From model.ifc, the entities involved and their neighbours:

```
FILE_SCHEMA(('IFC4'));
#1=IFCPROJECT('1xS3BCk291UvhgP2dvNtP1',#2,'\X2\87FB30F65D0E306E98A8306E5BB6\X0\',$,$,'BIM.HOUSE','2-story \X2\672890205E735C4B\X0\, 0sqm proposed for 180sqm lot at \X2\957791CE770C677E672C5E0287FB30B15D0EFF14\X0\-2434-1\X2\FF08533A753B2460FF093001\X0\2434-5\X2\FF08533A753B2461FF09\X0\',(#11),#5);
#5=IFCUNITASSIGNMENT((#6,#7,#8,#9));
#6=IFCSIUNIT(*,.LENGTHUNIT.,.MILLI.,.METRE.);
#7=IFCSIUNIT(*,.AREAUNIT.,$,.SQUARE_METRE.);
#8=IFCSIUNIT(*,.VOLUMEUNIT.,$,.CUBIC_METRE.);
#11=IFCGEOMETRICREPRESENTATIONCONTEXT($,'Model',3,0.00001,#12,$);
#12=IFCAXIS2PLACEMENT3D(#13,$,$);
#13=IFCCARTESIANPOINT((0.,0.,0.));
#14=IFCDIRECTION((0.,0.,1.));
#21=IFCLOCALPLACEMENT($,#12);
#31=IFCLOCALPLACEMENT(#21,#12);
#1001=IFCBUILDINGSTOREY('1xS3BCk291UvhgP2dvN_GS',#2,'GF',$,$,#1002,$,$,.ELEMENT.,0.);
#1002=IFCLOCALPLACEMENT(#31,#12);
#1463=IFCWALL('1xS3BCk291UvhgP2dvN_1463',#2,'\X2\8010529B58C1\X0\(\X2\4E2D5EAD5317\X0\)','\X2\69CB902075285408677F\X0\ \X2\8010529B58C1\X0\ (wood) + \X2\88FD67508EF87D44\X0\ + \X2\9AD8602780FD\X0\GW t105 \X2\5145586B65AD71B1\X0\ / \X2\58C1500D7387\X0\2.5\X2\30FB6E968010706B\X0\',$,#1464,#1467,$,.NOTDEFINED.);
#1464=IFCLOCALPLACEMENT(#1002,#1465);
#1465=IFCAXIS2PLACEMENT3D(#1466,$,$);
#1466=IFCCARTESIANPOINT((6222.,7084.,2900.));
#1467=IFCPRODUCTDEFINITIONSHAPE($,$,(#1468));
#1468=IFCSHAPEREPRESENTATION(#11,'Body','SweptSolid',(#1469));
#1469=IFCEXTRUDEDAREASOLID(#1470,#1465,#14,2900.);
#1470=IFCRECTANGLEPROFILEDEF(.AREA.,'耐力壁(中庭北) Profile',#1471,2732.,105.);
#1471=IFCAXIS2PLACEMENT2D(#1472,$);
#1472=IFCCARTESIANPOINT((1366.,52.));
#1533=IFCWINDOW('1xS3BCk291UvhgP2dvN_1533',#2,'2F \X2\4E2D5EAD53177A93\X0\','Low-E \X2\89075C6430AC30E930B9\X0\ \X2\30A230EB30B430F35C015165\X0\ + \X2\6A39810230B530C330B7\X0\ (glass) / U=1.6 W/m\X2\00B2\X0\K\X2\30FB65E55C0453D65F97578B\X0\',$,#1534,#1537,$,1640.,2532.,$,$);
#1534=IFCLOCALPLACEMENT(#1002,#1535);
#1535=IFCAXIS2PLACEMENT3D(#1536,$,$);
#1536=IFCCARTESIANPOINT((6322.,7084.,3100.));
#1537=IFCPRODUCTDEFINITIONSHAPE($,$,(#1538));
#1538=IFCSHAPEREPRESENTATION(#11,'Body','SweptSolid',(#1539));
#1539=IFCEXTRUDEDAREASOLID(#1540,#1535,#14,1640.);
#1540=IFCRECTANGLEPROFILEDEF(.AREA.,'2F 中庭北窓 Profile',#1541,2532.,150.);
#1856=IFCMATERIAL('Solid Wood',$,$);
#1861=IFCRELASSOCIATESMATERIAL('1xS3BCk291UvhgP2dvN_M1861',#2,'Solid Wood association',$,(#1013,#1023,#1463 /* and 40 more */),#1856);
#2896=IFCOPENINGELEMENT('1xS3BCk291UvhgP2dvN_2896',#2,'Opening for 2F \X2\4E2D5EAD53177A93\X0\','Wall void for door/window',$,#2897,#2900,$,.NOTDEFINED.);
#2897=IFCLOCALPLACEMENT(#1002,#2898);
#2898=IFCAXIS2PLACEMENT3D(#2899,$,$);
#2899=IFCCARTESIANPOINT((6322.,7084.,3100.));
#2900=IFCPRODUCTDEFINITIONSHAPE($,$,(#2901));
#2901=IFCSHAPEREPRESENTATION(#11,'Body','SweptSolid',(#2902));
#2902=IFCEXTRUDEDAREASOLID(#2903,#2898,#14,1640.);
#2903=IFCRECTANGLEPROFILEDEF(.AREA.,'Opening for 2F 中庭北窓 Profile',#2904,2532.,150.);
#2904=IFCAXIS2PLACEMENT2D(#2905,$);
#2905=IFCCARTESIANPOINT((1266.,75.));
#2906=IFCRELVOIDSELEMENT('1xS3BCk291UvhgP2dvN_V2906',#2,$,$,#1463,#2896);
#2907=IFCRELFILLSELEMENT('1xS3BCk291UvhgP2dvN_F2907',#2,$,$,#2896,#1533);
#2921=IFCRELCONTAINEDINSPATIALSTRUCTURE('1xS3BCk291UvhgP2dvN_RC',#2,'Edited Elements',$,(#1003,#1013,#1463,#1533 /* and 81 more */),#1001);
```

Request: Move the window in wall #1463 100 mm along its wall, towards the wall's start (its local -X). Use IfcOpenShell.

```python
import ifcopenshell
import ifcopenshell.api.geometry
import ifcopenshell.util.placement
import ifcopenshell.util.unit

model = ifcopenshell.open("model.ifc")
unit_scale = ifcopenshell.util.unit.calculate_unit_scale(model)

window = model.by_guid("1xS3BCk291UvhgP2dvN_1533")
opening = window.FillsVoids[0].RelatingOpeningElement
wall = opening.VoidsElements[0].RelatingBuildingElement

wall_matrix = ifcopenshell.util.placement.get_local_placement(wall.ObjectPlacement)
shift = wall_matrix[:3, 0] * -0.1 / unit_scale
before = ifcopenshell.util.placement.get_local_placement(window.ObjectPlacement)[:3, 3].copy()

# The window is not placed relative to its opening, so move both.
for product in (opening, window):
    matrix = ifcopenshell.util.placement.get_local_placement(product.ObjectPlacement)
    matrix[:3, 3] += shift
    ifcopenshell.api.geometry.edit_object_placement(model, product=product, matrix=matrix, is_si=False)

after = ifcopenshell.util.placement.get_local_placement(window.ObjectPlacement)[:3, 3]
print("window moved by", (after - before).round(3) + 0.0)

model.write("model-out.ifc")
```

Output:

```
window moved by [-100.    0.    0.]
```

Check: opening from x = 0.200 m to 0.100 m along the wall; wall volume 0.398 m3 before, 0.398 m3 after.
